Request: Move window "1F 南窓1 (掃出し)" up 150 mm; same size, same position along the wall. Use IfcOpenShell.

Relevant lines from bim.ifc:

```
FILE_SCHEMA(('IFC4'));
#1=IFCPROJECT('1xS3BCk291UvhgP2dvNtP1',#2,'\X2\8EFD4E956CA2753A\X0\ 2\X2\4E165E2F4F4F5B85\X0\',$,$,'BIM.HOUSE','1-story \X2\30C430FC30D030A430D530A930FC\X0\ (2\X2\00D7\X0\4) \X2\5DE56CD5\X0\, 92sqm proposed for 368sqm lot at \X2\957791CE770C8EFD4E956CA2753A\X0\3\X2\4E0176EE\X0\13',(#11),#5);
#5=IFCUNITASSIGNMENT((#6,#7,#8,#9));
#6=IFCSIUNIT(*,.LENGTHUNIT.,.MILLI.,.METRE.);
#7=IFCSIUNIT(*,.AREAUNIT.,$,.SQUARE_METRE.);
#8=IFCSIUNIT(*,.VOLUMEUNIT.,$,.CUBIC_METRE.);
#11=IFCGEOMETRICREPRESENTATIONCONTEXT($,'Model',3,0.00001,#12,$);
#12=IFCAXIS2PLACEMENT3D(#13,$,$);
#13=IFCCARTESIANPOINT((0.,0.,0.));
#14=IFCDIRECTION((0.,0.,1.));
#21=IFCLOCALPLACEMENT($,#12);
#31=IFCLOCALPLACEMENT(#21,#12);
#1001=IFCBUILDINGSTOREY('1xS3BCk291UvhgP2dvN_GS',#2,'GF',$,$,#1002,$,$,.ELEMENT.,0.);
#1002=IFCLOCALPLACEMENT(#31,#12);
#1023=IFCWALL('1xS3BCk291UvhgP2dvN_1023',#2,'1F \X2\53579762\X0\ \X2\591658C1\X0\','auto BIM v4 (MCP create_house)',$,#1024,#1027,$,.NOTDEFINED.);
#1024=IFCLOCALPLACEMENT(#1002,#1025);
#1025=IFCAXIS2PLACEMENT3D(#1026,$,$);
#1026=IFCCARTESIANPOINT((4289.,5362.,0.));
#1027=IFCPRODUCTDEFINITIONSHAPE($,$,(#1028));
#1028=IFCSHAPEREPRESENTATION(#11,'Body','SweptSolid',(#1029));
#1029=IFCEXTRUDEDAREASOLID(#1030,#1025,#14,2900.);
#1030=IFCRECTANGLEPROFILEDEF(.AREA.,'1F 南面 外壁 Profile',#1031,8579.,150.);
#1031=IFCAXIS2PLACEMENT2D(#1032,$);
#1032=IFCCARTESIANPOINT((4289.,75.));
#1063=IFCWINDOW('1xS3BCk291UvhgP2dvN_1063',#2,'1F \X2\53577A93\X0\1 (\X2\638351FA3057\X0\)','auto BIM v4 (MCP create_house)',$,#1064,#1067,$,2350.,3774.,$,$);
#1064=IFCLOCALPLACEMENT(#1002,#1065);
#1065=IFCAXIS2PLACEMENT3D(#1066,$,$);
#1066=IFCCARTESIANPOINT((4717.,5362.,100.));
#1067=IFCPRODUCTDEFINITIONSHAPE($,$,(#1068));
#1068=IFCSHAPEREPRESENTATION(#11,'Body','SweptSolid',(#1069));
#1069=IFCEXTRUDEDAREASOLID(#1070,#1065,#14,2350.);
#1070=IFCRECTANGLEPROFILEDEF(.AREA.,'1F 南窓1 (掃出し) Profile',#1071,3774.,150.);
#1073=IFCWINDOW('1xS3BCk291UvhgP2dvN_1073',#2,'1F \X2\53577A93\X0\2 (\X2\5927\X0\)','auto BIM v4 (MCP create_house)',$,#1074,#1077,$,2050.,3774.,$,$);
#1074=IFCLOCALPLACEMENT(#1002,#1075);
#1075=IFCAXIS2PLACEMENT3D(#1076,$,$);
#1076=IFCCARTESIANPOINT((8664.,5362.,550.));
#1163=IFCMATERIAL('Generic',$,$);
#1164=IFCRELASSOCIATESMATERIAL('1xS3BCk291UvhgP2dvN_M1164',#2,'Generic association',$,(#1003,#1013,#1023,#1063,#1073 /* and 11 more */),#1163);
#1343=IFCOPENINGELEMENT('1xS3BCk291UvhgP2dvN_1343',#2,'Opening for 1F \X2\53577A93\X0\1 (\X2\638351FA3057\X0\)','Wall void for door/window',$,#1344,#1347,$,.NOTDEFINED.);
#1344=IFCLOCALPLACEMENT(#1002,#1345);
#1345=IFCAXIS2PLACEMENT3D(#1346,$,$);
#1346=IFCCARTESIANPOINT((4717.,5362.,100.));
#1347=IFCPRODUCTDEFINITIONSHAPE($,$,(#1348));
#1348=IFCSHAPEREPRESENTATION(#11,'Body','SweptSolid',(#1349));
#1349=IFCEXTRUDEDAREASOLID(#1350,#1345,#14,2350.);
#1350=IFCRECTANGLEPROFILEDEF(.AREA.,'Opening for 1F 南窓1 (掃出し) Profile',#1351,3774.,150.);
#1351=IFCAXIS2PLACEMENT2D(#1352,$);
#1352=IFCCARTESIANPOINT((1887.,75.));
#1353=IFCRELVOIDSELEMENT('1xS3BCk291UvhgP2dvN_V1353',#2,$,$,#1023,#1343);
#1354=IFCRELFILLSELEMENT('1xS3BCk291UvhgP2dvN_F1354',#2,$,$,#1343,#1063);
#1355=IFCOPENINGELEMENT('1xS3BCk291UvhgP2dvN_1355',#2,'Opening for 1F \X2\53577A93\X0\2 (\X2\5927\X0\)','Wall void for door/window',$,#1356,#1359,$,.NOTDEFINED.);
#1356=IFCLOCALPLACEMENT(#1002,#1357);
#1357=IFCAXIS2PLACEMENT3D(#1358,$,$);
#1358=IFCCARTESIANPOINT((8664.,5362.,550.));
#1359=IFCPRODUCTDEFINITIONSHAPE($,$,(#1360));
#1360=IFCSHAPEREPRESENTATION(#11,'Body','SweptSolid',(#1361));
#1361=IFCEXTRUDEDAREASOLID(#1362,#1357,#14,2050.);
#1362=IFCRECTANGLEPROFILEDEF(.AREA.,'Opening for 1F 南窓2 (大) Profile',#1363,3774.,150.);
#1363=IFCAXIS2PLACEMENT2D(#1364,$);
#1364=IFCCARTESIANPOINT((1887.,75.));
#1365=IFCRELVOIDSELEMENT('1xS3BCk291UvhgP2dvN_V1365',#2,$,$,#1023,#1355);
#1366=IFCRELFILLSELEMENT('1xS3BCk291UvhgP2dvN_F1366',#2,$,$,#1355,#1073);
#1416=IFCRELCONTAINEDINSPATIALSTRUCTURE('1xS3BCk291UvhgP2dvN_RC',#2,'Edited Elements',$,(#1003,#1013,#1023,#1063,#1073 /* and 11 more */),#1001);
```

```python
import numpy as np
import ifcopenshell
import ifcopenshell.api.geometry
import ifcopenshell.util.placement
import ifcopenshell.util.unit

model = ifcopenshell.open("bim.ifc")
unit_scale = ifcopenshell.util.unit.calculate_unit_scale(model)

window = model.by_guid("1xS3BCk291UvhgP2dvN_1063")
opening = window.FillsVoids[0].RelatingOpeningElement
dz = 0.15 / unit_scale

shift = np.array([0.0, 0.0, dz])
# The window is not placed relative to its opening, so move both.
for product in (opening, window):
    matrix = ifcopenshell.util.placement.get_local_placement(product.ObjectPlacement)
    matrix[:3, 3] += shift
    ifcopenshell.api.geometry.edit_object_placement(model, product=product, matrix=matrix, is_si=False)

print(f"moved by {dz * unit_scale:+.3f} m")

model.write("bim_rev.ifc")
```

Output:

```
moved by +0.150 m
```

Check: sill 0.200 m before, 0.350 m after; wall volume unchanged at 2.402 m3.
